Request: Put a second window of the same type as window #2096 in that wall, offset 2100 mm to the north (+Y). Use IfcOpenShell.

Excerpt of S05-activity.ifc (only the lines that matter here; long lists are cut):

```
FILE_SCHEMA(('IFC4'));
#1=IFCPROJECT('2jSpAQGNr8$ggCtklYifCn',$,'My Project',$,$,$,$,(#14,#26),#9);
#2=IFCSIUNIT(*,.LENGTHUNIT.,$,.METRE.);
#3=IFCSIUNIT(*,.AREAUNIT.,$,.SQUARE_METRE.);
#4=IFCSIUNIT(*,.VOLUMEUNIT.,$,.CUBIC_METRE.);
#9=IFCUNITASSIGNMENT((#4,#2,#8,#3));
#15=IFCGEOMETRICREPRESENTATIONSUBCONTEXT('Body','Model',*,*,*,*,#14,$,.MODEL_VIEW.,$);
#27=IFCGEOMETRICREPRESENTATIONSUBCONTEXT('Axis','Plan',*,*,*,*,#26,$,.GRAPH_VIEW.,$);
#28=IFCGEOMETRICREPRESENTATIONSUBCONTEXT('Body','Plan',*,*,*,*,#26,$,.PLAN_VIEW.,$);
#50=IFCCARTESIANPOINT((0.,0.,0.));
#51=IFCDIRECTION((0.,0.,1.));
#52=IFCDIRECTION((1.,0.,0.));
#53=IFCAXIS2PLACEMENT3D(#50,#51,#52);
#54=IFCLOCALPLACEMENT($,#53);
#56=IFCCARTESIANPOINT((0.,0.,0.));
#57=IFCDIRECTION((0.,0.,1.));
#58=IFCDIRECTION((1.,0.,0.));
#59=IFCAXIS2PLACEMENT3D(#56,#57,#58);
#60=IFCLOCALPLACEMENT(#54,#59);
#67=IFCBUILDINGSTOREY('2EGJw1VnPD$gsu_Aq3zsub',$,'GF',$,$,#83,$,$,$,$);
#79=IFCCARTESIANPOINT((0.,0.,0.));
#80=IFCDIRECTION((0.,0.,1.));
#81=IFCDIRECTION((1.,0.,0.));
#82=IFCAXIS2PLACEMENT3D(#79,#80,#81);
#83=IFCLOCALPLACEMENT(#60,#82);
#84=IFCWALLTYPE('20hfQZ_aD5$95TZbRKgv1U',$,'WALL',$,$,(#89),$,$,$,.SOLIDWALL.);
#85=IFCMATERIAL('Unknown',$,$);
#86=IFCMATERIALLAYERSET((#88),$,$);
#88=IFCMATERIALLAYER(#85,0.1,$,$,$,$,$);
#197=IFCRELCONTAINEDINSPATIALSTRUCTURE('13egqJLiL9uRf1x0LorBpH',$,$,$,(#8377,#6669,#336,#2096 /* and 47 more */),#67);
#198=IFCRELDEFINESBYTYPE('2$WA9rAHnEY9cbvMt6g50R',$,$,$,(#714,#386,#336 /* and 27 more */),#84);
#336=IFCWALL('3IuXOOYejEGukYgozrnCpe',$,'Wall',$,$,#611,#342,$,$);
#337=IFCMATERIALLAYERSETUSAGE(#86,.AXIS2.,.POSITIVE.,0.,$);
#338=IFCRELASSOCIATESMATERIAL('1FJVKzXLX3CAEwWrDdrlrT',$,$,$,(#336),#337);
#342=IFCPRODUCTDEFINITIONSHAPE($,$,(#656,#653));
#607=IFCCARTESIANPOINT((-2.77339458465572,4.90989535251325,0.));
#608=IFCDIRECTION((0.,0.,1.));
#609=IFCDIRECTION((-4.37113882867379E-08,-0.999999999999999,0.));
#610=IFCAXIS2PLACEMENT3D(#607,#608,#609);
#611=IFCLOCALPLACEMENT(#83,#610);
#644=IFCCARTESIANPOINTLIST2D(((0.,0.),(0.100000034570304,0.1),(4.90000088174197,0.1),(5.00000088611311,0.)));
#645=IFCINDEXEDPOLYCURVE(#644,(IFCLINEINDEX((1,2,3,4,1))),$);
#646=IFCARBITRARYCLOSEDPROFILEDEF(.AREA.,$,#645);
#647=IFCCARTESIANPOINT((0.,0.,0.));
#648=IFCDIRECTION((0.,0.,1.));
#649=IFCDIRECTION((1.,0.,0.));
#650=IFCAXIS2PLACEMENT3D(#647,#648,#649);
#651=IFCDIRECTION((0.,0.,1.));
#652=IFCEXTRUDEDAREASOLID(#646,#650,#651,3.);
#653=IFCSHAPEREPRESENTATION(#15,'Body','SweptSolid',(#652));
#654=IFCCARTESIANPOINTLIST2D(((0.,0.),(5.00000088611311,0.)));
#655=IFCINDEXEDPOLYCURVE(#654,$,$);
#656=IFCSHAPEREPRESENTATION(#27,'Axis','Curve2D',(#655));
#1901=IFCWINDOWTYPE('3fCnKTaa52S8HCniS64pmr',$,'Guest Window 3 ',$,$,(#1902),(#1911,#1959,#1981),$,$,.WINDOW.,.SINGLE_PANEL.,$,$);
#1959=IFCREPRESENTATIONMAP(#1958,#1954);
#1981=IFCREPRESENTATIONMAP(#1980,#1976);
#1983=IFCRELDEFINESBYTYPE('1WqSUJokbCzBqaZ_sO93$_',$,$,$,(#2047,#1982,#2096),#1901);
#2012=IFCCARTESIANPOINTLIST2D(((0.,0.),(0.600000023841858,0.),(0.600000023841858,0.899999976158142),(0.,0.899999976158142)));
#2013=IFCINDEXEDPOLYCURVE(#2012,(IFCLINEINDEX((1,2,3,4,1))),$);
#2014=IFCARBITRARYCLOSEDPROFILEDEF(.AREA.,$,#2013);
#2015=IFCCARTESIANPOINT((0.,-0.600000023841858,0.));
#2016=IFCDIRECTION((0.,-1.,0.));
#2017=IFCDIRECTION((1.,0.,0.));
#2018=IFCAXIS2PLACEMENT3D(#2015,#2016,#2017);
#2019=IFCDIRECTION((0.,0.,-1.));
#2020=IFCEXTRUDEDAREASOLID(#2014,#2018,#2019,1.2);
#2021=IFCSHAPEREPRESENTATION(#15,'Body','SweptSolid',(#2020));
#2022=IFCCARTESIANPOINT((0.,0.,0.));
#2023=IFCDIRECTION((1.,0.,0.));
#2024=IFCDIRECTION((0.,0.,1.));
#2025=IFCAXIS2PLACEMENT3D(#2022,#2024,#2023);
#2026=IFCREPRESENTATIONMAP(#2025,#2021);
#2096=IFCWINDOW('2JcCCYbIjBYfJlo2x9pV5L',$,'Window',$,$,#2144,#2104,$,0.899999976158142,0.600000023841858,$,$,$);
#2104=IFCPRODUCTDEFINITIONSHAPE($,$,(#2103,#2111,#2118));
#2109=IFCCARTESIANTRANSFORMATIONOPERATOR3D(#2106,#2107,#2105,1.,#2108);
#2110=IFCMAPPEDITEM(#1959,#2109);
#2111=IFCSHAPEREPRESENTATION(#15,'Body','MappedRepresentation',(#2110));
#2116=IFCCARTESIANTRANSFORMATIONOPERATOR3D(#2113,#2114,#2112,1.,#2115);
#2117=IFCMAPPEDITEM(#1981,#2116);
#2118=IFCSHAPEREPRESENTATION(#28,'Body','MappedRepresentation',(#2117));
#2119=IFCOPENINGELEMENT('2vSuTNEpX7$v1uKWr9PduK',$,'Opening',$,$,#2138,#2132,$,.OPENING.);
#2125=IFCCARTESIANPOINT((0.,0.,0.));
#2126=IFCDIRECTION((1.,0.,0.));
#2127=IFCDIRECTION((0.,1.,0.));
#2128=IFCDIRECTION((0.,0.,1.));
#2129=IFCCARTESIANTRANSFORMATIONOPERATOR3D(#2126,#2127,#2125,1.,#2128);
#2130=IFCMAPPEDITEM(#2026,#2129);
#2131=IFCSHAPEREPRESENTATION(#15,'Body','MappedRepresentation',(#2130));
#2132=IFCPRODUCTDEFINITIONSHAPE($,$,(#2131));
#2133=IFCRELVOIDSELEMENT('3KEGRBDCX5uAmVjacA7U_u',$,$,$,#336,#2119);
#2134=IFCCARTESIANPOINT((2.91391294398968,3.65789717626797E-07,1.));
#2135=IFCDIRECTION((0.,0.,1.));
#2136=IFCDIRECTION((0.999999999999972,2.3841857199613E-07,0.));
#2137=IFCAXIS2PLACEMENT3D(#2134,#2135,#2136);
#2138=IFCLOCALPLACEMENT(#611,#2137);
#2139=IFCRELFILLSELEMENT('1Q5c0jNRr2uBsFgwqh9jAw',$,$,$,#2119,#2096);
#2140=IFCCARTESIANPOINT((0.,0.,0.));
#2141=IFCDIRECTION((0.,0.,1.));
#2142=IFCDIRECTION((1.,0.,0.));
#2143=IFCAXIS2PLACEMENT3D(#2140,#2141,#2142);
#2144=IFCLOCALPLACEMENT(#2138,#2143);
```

```python
import ifcopenshell
import ifcopenshell.api.feature
import ifcopenshell.api.geometry
import ifcopenshell.api.root
import ifcopenshell.geom
import ifcopenshell.util.element
import ifcopenshell.util.placement
import ifcopenshell.util.shape
import ifcopenshell.util.unit

model = ifcopenshell.open("S05-activity.ifc")
unit_scale = ifcopenshell.util.unit.calculate_unit_scale(model)
settings = ifcopenshell.geom.settings()


def volume(element):
    """Net volume in cubic metres, openings subtracted."""
    shape = ifcopenshell.geom.create_shape(settings, element)
    return ifcopenshell.util.shape.get_volume(shape.geometry)


window = model.by_id(2096)
opening = window.FillsVoids[0].RelatingOpeningElement
wall = opening.VoidsElements[0].RelatingBuildingElement
before = volume(wall)
shift = ifcopenshell.util.placement.get_local_placement(wall.ObjectPlacement)[:3, 0] * -2.1 / unit_scale

# copy_class copies the void relationship, type, container and properties, but no geometry.
new_opening = ifcopenshell.api.root.copy_class(model, product=opening)
new_opening.Representation = ifcopenshell.util.element.copy_deep(
    model, opening.Representation, exclude=["IfcGeometricRepresentationContext", "IfcRepresentationMap"]
)
new_window = ifcopenshell.api.root.copy_class(model, product=window)
new_window.Representation = ifcopenshell.util.element.copy_deep(
    model, window.Representation, exclude=["IfcGeometricRepresentationContext", "IfcRepresentationMap"]
)
ifcopenshell.api.feature.add_filling(model, opening=new_opening, element=new_window)

for old, new in ((opening, new_opening), (window, new_window)):
    matrix = ifcopenshell.util.placement.get_local_placement(old.ObjectPlacement)
    matrix[:3, 3] += shift
    ifcopenshell.api.geometry.edit_object_placement(model, product=new, matrix=matrix, is_si=False)

after = volume(wall)

print(f"wall volume {before:.3f} -> {after:.3f} m3")

model.write("S05-activity_v2.ifc")
```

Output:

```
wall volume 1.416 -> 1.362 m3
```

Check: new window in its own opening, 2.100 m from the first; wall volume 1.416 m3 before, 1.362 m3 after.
